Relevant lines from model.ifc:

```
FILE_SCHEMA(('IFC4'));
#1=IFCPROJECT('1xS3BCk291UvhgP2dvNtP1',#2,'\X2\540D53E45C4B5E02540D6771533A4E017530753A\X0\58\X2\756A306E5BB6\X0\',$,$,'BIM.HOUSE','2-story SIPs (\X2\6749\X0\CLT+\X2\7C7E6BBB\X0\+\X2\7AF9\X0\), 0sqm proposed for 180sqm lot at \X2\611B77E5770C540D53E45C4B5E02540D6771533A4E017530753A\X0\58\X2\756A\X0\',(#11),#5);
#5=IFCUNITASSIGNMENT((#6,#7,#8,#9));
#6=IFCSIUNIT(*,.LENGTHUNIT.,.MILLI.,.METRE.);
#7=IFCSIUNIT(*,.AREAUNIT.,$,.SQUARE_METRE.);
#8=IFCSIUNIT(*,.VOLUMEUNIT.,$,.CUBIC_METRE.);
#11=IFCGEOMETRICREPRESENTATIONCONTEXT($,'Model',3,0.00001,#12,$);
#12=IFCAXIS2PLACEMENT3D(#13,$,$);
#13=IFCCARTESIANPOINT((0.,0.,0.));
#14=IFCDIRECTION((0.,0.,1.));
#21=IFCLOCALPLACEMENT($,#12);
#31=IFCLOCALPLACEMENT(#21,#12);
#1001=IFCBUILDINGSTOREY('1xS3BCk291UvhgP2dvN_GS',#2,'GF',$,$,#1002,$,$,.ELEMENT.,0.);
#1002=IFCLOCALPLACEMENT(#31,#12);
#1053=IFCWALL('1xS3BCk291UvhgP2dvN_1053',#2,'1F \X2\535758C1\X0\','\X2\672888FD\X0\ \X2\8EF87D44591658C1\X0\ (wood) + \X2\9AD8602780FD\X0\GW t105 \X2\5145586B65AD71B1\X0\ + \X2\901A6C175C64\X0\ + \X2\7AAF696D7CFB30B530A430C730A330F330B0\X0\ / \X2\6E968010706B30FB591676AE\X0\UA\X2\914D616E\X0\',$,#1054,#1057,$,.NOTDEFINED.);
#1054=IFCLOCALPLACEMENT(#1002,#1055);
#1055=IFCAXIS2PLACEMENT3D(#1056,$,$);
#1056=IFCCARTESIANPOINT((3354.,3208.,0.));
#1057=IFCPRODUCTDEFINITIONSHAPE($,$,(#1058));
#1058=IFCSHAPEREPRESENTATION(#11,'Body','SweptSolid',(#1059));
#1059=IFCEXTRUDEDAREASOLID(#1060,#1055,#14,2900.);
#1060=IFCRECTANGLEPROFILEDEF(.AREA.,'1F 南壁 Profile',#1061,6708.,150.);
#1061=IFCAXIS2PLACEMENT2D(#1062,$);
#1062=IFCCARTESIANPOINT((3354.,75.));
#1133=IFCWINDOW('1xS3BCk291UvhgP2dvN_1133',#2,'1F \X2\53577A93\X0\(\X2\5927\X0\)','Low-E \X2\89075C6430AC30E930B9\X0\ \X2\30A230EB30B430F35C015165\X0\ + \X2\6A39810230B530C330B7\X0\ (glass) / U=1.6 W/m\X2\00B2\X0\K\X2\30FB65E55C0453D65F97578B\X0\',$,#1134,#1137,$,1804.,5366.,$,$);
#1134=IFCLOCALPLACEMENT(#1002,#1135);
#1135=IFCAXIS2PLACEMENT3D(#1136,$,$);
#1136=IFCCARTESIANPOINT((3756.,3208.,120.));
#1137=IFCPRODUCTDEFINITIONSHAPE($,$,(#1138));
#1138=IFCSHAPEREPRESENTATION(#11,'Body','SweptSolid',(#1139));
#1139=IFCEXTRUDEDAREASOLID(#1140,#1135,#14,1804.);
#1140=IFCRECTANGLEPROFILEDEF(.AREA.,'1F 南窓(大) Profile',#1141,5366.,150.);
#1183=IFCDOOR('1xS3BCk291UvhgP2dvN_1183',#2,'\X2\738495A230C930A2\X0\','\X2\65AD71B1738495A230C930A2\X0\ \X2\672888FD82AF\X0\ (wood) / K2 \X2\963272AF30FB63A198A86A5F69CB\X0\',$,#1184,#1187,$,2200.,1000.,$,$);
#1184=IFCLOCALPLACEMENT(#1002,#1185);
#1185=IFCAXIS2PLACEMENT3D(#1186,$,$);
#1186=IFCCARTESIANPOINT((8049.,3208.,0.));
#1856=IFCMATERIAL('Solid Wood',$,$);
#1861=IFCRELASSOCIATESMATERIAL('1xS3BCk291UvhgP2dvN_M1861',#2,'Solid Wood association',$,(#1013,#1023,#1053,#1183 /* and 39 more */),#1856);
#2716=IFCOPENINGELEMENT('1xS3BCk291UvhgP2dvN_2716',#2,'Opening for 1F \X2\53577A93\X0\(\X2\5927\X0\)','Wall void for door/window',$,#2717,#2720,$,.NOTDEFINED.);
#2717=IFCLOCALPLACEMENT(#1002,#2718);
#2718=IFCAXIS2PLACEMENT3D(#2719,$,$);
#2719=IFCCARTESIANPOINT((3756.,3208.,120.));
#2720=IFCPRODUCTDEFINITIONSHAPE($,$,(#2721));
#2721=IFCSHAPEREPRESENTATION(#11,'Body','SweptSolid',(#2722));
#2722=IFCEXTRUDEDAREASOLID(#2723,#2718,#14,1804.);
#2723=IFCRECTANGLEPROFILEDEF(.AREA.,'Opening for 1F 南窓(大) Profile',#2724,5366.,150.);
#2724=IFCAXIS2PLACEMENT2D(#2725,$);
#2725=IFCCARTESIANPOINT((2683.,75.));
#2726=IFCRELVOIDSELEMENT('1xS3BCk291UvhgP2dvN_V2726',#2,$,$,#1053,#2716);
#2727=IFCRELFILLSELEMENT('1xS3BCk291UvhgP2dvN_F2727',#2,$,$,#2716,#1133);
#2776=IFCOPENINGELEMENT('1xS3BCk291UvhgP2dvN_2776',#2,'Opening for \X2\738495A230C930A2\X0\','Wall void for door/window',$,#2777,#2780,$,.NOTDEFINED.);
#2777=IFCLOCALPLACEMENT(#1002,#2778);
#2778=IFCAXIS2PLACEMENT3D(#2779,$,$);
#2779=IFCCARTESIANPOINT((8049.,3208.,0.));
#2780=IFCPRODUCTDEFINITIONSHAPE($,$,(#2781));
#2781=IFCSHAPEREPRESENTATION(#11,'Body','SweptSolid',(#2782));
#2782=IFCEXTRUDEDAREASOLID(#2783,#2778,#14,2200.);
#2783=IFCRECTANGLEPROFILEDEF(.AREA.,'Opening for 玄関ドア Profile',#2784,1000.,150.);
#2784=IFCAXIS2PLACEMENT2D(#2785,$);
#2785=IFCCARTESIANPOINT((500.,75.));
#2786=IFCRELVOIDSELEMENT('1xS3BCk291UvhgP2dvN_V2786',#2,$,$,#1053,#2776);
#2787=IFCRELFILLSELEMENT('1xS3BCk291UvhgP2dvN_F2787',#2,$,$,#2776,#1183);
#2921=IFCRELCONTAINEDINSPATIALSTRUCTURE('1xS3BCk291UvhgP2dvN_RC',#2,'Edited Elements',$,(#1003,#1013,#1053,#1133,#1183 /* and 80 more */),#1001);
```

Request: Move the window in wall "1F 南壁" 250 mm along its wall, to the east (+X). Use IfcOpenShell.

```python
import ifcopenshell
import ifcopenshell.api.geometry
import ifcopenshell.util.placement

model = ifcopenshell.open("model.ifc")

window = model.by_id(1133)
opening = window.FillsVoids[0].RelatingOpeningElement
wall = opening.VoidsElements[0].RelatingBuildingElement

wall_matrix = ifcopenshell.util.placement.get_local_placement(wall.ObjectPlacement)
shift = wall_matrix[:3, 0] * 250.0
before = ifcopenshell.util.placement.get_local_placement(window.ObjectPlacement)[:3, 3].copy()

# The window is not placed relative to its opening, so move both.
for product in (opening, window):
    matrix = ifcopenshell.util.placement.get_local_placement(product.ObjectPlacement)
    matrix[:3, 3] += shift
    ifcopenshell.api.geometry.edit_object_placement(model, product=product, matrix=matrix, is_si=False)

after = ifcopenshell.util.placement.get_local_placement(window.ObjectPlacement)[:3, 3]
print("window moved by", (after - before).round(3) + 0.0)

model.write("model_updated.ifc")
```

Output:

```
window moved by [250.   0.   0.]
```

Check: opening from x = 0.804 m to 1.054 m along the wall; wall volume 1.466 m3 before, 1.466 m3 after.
